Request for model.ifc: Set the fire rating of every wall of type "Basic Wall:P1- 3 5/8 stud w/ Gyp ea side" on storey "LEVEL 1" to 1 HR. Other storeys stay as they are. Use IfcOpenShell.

First a look at what the model holds.

```python
import ifcopenshell
import ifcopenshell.util.element

model = ifcopenshell.open("model.ifc")
print(model.schema)
storey = next(s for s in model.by_type("IfcBuildingStorey") if s.Name == "LEVEL 1")
walls = [e for e in ifcopenshell.util.element.get_decomposition(storey) if e.is_a("IfcWall")]
seen = {}
for e in walls:
    element_type = ifcopenshell.util.element.get_type(e)
    key = (element_type.Name if element_type != e and element_type else None, ifcopenshell.util.element.get_pset(e, "Pset_WallCommon", "FireRating"))
    seen[key] = seen.get(key, 0) + 1
for (name, value), count in sorted(seen.items(), key=str):
    print(count, "x", name, "|", value)
```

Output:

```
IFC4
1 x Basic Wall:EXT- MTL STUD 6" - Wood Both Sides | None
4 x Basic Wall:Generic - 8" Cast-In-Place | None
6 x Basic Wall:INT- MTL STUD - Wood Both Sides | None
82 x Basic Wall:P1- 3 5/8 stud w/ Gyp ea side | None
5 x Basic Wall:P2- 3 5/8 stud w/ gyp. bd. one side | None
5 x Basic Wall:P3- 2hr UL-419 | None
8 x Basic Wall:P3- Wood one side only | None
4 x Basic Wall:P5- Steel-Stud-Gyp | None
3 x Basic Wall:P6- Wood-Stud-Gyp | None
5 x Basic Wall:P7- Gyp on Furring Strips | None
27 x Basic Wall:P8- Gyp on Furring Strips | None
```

```python
import ifcopenshell
import ifcopenshell.api.pset
import ifcopenshell.util.element

model = ifcopenshell.open("model.ifc")

storey = next(s for s in model.by_type("IfcBuildingStorey") if s.Name == "LEVEL 1")
walls = [e for e in ifcopenshell.util.element.get_decomposition(storey) if e.is_a("IfcWall")]

count = 0
for e in walls:
    element_type = ifcopenshell.util.element.get_type(e)
    if element_type in (None, e) or element_type.Name != "Basic Wall:P1- 3 5/8 stud w/ Gyp ea side":
        continue
    # add_pset returns the element's existing set when there is one.
    pset = ifcopenshell.api.pset.add_pset(model, product=e, name="Pset_WallCommon")
    ifcopenshell.api.pset.edit_pset(model, pset=pset, properties={"FireRating": "1 HR"})
    count += 1

print(count, "walls updated")

model.write("model-out.ifc")
```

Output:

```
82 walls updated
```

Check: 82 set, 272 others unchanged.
